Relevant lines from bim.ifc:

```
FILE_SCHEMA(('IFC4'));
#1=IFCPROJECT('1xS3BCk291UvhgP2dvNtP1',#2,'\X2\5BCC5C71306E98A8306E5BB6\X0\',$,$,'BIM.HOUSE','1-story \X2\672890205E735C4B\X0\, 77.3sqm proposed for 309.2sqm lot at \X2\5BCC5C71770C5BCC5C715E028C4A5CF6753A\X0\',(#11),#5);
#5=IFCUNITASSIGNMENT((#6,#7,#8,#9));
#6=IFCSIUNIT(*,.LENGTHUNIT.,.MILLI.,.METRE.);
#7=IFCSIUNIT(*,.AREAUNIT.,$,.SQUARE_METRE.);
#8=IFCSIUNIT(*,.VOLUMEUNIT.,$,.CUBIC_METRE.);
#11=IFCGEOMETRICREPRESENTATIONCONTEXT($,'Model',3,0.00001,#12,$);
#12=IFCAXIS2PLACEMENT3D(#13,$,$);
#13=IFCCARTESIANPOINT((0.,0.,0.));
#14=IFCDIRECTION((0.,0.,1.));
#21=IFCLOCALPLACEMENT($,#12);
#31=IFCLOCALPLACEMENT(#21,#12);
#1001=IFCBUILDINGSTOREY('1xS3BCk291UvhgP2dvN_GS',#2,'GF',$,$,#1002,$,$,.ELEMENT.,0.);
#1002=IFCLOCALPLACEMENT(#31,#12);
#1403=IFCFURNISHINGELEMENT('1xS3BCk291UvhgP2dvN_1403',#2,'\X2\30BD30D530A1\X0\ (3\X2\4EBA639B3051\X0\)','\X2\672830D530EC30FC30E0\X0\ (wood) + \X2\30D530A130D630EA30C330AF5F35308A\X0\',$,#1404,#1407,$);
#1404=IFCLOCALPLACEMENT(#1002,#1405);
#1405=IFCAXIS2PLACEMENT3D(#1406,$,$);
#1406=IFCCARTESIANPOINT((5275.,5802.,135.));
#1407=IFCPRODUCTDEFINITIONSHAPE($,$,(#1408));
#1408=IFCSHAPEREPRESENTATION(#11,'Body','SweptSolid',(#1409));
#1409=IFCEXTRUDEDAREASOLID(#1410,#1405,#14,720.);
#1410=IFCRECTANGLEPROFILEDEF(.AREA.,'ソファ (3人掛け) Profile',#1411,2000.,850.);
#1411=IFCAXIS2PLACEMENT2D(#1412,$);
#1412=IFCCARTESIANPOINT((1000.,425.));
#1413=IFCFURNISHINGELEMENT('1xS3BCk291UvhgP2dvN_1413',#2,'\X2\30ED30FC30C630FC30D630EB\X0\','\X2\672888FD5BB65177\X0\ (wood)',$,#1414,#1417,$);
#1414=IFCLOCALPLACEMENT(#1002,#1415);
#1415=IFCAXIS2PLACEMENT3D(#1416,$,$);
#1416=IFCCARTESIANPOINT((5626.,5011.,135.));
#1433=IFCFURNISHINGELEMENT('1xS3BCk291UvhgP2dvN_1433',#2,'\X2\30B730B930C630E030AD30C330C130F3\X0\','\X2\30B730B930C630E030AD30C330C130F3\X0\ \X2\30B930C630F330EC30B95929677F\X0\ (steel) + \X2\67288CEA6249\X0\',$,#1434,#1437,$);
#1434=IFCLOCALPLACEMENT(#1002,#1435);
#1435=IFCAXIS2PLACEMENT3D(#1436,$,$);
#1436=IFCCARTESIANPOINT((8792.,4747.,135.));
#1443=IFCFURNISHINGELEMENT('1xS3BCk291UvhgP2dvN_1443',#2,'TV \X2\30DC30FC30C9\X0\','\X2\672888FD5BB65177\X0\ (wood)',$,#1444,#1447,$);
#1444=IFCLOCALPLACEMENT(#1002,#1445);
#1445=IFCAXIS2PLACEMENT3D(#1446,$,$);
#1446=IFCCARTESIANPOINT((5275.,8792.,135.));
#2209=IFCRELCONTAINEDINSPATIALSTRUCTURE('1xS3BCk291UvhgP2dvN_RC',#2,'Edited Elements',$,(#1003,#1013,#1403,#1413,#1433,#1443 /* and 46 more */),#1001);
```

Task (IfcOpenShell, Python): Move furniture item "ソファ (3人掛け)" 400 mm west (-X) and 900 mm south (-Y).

```python
import ifcopenshell
import ifcopenshell.api.geometry
import ifcopenshell.util.placement
import ifcopenshell.util.unit

model = ifcopenshell.open("bim.ifc")
unit_scale = ifcopenshell.util.unit.calculate_unit_scale(model)

item = model.by_guid("1xS3BCk291UvhgP2dvN_1403")
matrix = ifcopenshell.util.placement.get_local_placement(item.ObjectPlacement)
matrix[0, 3] -= 0.4 / unit_scale
matrix[1, 3] -= 0.9 / unit_scale
ifcopenshell.api.geometry.edit_object_placement(model, product=item, matrix=matrix, is_si=False)

print(ifcopenshell.util.placement.get_local_placement(item.ObjectPlacement).round(3) + 0.0)

model.write("bim_updated.ifc")
```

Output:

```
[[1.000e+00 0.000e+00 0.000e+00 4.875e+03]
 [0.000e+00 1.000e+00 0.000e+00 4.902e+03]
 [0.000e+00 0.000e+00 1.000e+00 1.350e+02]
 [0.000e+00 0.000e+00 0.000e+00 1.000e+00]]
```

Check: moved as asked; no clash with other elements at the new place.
